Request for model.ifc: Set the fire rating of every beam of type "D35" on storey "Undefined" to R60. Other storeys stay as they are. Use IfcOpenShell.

First a look at what the model holds.

```python
import ifcopenshell
import ifcopenshell.util.element

model = ifcopenshell.open("model.ifc")
print(model.schema)
storey = next(s for s in model.by_type("IfcBuildingStorey") if s.Name == "Undefined")
beams = [e for e in ifcopenshell.util.element.get_decomposition(storey) if e.is_a("IfcBeam")]
seen = {}
for e in beams:
    element_type = ifcopenshell.util.element.get_type(e)
    key = (element_type.Name if element_type != e and element_type else None, ifcopenshell.util.element.get_pset(e, "Pset_BeamCommon", "FireRating"))
    seen[key] = seen.get(key, 0) + 1
for (name, value), count in sorted(seen.items(), key=str):
    print(count, "x", name, "|", value)
```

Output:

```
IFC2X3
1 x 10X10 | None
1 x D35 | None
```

```python
import ifcopenshell
import ifcopenshell.api.pset
import ifcopenshell.util.element

model = ifcopenshell.open("model.ifc")

storey = next(s for s in model.by_type("IfcBuildingStorey") if s.Name == "Undefined")
beams = [e for e in ifcopenshell.util.element.get_decomposition(storey) if e.is_a("IfcBeam")]

count = 0
for e in beams:
    element_type = ifcopenshell.util.element.get_type(e)
    if element_type in (None, e) or element_type.Name != "D35":
        continue
    # add_pset returns the element's existing set when there is one.
    pset = ifcopenshell.api.pset.add_pset(model, product=e, name="Pset_BeamCommon")
    ifcopenshell.api.pset.edit_pset(model, pset=pset, properties={"FireRating": "R60"})
    count += 1

print(count, "beams updated")

model.write("model_edited.ifc")
```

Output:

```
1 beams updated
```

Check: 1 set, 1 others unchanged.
